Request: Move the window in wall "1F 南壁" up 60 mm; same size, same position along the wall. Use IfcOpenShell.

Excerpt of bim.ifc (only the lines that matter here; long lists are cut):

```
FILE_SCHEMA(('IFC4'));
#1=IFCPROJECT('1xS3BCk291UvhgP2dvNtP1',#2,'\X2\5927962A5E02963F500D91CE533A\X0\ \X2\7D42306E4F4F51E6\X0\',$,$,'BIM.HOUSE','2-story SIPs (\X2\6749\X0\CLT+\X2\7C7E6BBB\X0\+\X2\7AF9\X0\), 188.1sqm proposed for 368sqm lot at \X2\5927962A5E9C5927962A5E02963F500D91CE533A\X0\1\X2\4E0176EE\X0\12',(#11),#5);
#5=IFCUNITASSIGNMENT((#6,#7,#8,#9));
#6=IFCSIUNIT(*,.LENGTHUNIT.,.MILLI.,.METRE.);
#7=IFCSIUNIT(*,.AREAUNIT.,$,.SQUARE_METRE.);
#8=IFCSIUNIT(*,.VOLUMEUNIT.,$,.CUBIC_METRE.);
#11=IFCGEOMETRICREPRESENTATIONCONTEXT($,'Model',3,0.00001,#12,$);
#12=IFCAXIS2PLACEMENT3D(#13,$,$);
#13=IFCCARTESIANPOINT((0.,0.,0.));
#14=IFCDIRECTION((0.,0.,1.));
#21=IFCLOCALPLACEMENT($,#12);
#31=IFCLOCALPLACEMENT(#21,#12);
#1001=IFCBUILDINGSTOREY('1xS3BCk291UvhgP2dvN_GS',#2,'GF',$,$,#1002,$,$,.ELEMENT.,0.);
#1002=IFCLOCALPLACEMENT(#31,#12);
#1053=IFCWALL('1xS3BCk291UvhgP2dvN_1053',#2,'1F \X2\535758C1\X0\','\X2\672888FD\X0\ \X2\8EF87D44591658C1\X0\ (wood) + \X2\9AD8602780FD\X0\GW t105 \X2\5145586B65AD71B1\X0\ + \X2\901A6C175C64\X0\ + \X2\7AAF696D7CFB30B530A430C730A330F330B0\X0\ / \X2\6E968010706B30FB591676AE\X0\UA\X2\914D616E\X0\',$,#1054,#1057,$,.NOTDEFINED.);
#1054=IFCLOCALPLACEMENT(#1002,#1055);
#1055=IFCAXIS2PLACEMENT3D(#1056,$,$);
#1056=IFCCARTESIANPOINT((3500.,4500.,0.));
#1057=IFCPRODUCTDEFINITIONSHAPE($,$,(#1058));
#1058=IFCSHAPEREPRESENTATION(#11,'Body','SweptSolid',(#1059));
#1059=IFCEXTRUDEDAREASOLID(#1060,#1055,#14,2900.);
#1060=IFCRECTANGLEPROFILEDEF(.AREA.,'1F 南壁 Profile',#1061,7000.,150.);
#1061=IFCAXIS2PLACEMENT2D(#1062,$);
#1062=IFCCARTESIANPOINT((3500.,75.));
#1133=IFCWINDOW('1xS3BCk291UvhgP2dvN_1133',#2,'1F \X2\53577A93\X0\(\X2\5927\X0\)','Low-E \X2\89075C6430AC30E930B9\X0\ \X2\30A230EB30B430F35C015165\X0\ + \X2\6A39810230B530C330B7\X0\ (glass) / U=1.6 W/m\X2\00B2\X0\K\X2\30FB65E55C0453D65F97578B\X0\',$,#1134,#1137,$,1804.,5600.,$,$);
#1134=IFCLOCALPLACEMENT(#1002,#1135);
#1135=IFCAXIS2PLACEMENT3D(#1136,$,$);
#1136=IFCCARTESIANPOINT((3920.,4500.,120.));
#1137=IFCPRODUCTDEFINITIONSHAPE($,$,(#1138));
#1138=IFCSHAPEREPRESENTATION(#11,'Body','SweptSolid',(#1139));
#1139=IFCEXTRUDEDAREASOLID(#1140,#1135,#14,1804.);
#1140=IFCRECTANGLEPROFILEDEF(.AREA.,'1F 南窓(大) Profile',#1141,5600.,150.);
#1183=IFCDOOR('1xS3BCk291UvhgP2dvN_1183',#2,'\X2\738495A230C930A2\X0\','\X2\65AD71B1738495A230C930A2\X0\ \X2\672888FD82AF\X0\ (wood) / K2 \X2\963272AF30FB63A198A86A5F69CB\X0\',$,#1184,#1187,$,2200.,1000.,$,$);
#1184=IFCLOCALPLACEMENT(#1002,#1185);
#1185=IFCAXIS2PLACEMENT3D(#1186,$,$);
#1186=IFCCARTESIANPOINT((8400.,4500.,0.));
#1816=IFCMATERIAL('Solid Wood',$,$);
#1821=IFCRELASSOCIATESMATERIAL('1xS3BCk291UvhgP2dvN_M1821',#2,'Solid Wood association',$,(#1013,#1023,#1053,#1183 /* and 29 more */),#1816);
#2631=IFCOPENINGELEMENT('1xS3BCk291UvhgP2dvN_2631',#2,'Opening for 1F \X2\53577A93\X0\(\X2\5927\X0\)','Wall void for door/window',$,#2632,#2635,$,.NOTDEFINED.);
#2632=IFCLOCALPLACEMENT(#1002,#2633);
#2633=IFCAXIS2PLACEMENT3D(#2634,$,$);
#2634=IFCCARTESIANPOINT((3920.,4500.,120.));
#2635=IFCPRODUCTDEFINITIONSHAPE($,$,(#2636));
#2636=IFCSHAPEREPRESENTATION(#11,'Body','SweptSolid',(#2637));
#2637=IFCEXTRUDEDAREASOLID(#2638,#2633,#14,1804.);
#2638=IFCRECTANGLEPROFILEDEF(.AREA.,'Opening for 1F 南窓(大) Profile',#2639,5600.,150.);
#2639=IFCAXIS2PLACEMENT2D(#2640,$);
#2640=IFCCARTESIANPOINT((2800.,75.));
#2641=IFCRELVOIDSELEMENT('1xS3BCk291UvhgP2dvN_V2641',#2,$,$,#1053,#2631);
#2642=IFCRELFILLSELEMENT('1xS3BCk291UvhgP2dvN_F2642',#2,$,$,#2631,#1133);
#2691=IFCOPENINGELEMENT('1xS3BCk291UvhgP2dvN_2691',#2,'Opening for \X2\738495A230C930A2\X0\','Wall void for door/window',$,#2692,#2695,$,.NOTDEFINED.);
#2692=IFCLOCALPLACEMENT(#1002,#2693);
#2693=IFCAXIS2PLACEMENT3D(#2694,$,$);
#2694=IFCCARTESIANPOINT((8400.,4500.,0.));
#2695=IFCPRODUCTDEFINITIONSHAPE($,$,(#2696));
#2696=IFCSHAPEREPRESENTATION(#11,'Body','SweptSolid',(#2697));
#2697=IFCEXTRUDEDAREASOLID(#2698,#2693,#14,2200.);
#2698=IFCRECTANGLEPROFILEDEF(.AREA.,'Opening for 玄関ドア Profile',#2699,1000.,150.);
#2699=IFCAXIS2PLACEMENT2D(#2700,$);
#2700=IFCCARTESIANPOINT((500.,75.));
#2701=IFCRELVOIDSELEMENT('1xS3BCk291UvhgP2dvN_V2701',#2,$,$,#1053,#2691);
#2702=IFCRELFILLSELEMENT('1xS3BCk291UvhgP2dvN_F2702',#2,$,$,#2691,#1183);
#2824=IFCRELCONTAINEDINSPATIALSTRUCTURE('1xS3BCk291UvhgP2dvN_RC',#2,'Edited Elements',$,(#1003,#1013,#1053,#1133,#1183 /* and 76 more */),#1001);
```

```python
import numpy as np
import ifcopenshell
import ifcopenshell.api.geometry
import ifcopenshell.util.placement
import ifcopenshell.util.unit

model = ifcopenshell.open("bim.ifc")
unit_scale = ifcopenshell.util.unit.calculate_unit_scale(model)

window = model.by_id(1133)
opening = window.FillsVoids[0].RelatingOpeningElement
dz = 60.0

shift = np.array([0.0, 0.0, dz])
# The window is not placed relative to its opening, so move both.
for product in (opening, window):
    matrix = ifcopenshell.util.placement.get_local_placement(product.ObjectPlacement)
    matrix[:3, 3] += shift
    ifcopenshell.api.geometry.edit_object_placement(model, product=product, matrix=matrix, is_si=False)

print(f"moved by {dz * unit_scale:+.3f} m")

model.write("bim_rev.ifc")
```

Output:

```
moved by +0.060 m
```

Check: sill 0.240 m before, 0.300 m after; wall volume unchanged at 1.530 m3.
